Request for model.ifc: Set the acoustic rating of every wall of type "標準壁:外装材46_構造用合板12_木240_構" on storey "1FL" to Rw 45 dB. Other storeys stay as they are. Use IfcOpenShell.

First a look at what the model holds.

```python
import ifcopenshell
import ifcopenshell.util.element

model = ifcopenshell.open("model.ifc")
print(model.schema)
storey = next(s for s in model.by_type("IfcBuildingStorey") if s.Name == "1FL")
walls = [e for e in ifcopenshell.util.element.get_decomposition(storey) if e.is_a("IfcWall")]
seen = {}
for e in walls:
    element_type = ifcopenshell.util.element.get_type(e)
    key = (element_type.Name if element_type != e and element_type else None, ifcopenshell.util.element.get_pset(e, "Pset_WallCommon", "AcousticRating"))
    seen[key] = seen.get(key, 0) + 1
for (name, value), count in sorted(seen.items(), key=str):
    print(count, "x", name, "|", value)
```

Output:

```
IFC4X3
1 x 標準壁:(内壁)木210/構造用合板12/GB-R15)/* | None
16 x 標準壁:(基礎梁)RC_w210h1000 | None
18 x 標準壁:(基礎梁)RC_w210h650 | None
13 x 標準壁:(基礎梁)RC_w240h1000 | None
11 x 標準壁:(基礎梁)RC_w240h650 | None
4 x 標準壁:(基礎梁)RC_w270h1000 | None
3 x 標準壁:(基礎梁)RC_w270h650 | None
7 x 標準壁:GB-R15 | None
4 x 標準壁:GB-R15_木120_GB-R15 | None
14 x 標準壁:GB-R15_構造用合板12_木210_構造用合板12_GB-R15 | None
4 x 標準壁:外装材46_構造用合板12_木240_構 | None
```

```python
import ifcopenshell
import ifcopenshell.api.pset
import ifcopenshell.util.element

model = ifcopenshell.open("model.ifc")

storey = next(s for s in model.by_type("IfcBuildingStorey") if s.Name == "1FL")
walls = [e for e in ifcopenshell.util.element.get_decomposition(storey) if e.is_a("IfcWall")]

count = 0
for e in walls:
    element_type = ifcopenshell.util.element.get_type(e)
    if element_type in (None, e) or element_type.Name != "標準壁:外装材46_構造用合板12_木240_構":
        continue
    # add_pset returns the element's existing set when there is one.
    pset = ifcopenshell.api.pset.add_pset(model, product=e, name="Pset_WallCommon")
    ifcopenshell.api.pset.edit_pset(model, pset=pset, properties={"AcousticRating": "Rw 45 dB"})
    count += 1

print(count, "walls updated")

model.write("model_rev.ifc")
```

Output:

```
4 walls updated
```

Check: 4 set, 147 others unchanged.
